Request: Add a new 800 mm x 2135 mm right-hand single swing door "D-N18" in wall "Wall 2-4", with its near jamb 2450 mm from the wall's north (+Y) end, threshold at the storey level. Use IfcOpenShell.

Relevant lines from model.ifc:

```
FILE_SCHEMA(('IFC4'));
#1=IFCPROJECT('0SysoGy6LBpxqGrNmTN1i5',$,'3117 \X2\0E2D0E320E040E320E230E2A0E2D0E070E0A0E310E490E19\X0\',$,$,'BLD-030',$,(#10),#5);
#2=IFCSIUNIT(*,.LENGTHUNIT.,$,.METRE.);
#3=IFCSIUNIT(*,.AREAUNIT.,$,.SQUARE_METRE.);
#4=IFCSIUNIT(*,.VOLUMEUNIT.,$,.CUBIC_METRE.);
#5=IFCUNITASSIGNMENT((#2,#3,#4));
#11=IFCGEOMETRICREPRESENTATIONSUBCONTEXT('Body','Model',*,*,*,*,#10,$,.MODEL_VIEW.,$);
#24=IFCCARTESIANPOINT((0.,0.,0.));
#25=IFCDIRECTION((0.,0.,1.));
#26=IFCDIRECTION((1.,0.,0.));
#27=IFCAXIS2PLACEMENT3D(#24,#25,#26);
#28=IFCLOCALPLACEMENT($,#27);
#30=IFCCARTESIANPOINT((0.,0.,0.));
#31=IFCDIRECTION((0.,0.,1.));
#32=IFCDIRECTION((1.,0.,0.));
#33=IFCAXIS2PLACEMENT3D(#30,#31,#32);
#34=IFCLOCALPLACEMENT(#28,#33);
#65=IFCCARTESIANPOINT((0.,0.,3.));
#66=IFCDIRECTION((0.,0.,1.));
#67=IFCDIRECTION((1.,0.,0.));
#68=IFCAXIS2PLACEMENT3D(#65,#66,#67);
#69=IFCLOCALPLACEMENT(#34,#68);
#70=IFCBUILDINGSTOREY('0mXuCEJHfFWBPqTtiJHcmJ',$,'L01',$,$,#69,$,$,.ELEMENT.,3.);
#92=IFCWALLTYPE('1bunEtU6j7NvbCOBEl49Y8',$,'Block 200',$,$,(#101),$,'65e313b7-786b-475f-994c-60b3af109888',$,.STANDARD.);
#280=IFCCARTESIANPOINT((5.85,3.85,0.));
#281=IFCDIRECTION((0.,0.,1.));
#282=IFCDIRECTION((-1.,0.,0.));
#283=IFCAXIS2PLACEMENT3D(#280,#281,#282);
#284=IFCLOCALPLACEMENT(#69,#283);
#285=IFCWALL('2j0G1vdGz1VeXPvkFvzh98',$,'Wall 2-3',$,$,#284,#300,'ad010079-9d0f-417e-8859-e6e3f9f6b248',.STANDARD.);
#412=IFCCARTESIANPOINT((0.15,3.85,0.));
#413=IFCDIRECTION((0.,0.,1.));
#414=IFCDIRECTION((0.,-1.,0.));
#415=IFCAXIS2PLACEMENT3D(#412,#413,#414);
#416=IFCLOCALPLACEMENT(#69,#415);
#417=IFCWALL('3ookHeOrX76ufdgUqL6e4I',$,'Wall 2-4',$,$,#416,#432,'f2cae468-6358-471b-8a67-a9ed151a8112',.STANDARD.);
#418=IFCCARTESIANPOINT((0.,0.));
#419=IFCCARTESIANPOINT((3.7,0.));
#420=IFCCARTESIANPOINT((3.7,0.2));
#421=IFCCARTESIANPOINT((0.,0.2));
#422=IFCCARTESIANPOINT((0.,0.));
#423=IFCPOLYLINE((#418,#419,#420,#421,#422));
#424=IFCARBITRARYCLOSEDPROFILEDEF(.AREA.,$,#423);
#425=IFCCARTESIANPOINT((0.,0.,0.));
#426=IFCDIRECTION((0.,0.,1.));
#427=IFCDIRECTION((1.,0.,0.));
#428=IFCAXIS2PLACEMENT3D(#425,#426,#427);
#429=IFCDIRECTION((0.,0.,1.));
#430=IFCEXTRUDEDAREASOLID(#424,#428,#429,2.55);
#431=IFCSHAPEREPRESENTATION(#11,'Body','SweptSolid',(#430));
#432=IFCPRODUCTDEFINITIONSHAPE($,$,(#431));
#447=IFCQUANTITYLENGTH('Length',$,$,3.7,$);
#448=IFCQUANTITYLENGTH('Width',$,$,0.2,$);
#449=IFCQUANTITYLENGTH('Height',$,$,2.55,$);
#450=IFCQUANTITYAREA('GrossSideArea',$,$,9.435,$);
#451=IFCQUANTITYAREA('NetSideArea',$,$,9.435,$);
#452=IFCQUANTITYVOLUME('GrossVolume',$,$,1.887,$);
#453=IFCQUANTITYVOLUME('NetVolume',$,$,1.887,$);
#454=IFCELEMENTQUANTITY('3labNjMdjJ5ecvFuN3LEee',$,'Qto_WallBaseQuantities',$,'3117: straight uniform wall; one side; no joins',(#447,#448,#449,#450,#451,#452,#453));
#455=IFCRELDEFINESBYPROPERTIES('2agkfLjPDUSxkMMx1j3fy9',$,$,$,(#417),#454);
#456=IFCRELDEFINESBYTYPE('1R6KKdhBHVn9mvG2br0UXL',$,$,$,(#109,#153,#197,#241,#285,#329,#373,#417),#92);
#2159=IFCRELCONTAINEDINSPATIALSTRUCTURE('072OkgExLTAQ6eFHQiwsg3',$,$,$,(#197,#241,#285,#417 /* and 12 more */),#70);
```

```python
import numpy as np
import ifcopenshell
import ifcopenshell.api.feature
import ifcopenshell.api.geometry
import ifcopenshell.api.pset
import ifcopenshell.api.root
import ifcopenshell.api.spatial
import ifcopenshell.geom
import ifcopenshell.util.element
import ifcopenshell.util.placement
import ifcopenshell.util.representation
import ifcopenshell.util.shape
import ifcopenshell.util.unit

model = ifcopenshell.open("model.ifc")
unit_scale = ifcopenshell.util.unit.calculate_unit_scale(model)
area_scale = ifcopenshell.util.unit.calculate_unit_scale(model, "AREAUNIT")
volume_scale = ifcopenshell.util.unit.calculate_unit_scale(model, "VOLUMEUNIT")
settings = ifcopenshell.geom.settings()


def volume(element):
    """Net volume in cubic metres, openings subtracted."""
    shape = ifcopenshell.geom.create_shape(settings, element)
    return ifcopenshell.util.shape.get_volume(shape.geometry)


wall = model.by_guid("3ookHeOrX76ufdgUqL6e4I")
storey = ifcopenshell.util.element.get_container(wall, ifc_class="IfcBuildingStorey")
context = ifcopenshell.util.representation.get_context(model, "Model", "Body", "MODEL_VIEW")
before = volume(wall)

width, height, from_end, sill = 0.8, 2.135, 2.45, 0.0  # metres

# The wall runs along its own X axis, and the end named is its -X end.
wall_shape = ifcopenshell.geom.create_shape(settings, wall)
x, y, z = ifcopenshell.util.shape.get_vertices(wall_shape.geometry).T
start = x.min() + from_end
face, thickness = float(y.min()), float(y.max() - y.min())
wall_matrix = ifcopenshell.util.placement.get_local_placement(wall.ObjectPlacement)
level = ifcopenshell.util.placement.get_local_placement(storey.ObjectPlacement)[2, 3]


def in_wall(x, y):
    """Placement at x, y metres in the wall's axes, at sill height."""
    matrix = wall_matrix.copy()
    matrix[:, 3] = wall_matrix @ np.array([x / unit_scale, y / unit_scale, 0.0, 1.0])
    matrix[2, 3] = level + sill / unit_scale
    return matrix


# Opening: a box that overshoots both wall faces by 50 mm.
opening = ifcopenshell.api.root.create_entity(model, ifc_class="IfcOpeningElement", predefined_type="OPENING")
box = ifcopenshell.api.geometry.add_wall_representation(
    model, context=context, length=width, height=height, thickness=thickness + 0.1
)
ifcopenshell.api.geometry.assign_representation(model, product=opening, representation=box)
ifcopenshell.api.geometry.edit_object_placement(model, product=opening, matrix=in_wall(start, face - 0.05), is_si=False)
ifcopenshell.api.feature.add_feature(model, feature=opening, element=wall)

door = ifcopenshell.api.root.create_entity(model, ifc_class="IfcDoor", name="D-N18", predefined_type="DOOR")
door.OverallWidth, door.OverallHeight = width / unit_scale, height / unit_scale
door.OperationType = "SINGLE_SWING_RIGHT"
body = ifcopenshell.api.geometry.add_door_representation(
    model,
    context=context,
    overall_width=door.OverallWidth,
    overall_height=door.OverallHeight,
    operation_type="SINGLE_SWING_RIGHT",
    lining_properties={"LiningDepth": thickness / unit_scale, "ThresholdDepth": thickness / unit_scale},
)
ifcopenshell.api.geometry.assign_representation(model, product=door, representation=body)
ifcopenshell.api.spatial.assign_container(model, products=[door], relating_structure=storey)
ifcopenshell.api.feature.add_filling(model, opening=opening, element=door)

# The lining spans the wall, so the door starts at the wall face.
ifcopenshell.api.geometry.edit_object_placement(model, product=door, matrix=in_wall(start, face), is_si=False)

after = volume(wall)

# Update the wall's stored quantities.
qto = model.by_id(ifcopenshell.util.element.get_pset(wall, "Qto_WallBaseQuantities", should_inherit=False)["id"])
ifcopenshell.api.pset.edit_qto(model, qto=qto, properties={
    "NetSideArea": after / thickness / area_scale,
    "NetVolume": after / volume_scale,
})

print(f"wall volume {before:.3f} -> {after:.3f} m3")

model.write("model_updated.ifc")
```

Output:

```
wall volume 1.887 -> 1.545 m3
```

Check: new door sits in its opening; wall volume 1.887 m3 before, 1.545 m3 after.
